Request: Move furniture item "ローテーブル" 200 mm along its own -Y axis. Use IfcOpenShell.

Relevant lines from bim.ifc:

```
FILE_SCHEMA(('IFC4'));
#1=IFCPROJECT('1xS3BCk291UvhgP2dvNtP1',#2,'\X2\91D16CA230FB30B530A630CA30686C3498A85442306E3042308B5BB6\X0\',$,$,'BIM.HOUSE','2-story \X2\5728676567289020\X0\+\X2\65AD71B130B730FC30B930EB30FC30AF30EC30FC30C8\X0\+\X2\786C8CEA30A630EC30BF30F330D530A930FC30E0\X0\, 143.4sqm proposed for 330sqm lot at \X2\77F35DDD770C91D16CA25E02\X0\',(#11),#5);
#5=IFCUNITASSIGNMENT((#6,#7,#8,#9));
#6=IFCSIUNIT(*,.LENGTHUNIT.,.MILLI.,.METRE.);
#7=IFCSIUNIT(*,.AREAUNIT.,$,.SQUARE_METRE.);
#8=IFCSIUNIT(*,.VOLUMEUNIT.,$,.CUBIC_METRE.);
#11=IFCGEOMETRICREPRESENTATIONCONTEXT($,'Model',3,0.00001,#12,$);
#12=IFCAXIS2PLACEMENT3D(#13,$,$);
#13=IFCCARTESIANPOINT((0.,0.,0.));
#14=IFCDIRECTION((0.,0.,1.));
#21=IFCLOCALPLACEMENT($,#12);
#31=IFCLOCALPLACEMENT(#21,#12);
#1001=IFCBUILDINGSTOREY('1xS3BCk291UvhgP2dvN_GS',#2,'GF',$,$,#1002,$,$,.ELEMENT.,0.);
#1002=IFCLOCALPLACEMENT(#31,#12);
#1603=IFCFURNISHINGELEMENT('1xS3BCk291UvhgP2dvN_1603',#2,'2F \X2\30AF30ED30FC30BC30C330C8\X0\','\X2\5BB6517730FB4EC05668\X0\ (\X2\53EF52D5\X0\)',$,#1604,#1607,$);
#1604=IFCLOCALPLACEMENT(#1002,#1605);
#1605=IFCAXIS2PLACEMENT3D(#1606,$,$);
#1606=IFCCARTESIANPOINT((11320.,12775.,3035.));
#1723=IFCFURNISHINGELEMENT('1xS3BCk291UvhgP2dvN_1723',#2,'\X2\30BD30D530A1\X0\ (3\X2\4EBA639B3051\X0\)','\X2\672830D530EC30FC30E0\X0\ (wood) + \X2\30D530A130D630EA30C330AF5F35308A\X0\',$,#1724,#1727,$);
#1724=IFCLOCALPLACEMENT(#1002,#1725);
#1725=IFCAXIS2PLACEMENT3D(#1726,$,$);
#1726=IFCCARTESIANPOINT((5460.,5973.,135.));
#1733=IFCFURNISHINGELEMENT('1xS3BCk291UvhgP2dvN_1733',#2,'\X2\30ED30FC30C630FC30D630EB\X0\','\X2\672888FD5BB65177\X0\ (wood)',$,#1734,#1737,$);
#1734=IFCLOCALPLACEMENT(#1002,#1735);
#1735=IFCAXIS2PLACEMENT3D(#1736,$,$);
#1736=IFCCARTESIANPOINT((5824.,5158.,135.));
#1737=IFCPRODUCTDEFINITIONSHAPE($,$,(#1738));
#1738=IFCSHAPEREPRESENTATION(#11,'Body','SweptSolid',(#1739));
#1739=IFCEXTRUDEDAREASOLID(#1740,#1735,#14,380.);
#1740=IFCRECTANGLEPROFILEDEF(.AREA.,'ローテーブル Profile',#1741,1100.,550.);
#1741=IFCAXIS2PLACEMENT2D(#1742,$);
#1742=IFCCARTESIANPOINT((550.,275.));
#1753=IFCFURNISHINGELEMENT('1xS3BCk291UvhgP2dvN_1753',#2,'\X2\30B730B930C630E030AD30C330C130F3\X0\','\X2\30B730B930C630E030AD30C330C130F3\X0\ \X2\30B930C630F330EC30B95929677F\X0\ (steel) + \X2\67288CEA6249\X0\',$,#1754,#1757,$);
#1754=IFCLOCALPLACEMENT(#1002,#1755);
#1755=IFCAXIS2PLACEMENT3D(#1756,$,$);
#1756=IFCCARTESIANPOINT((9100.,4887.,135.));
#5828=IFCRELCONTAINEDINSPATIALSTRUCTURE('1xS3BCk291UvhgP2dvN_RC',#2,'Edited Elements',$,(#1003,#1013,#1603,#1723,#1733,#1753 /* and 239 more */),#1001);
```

```python
import ifcopenshell
import ifcopenshell.api.geometry
import ifcopenshell.util.placement
import ifcopenshell.util.unit

model = ifcopenshell.open("bim.ifc")
unit_scale = ifcopenshell.util.unit.calculate_unit_scale(model)

item = model.by_guid("1xS3BCk291UvhgP2dvN_1733")
matrix = ifcopenshell.util.placement.get_local_placement(item.ObjectPlacement)
matrix[:3, 3] -= matrix[:3, 1] * 0.2 / unit_scale
ifcopenshell.api.geometry.edit_object_placement(model, product=item, matrix=matrix, is_si=False)

print(ifcopenshell.util.placement.get_local_placement(item.ObjectPlacement).round(3) + 0.0)

model.write("bim_v2.ifc")
```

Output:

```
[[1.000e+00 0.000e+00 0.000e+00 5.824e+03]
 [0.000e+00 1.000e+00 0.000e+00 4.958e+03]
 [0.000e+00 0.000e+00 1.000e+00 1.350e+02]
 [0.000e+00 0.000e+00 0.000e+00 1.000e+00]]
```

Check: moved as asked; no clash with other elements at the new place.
